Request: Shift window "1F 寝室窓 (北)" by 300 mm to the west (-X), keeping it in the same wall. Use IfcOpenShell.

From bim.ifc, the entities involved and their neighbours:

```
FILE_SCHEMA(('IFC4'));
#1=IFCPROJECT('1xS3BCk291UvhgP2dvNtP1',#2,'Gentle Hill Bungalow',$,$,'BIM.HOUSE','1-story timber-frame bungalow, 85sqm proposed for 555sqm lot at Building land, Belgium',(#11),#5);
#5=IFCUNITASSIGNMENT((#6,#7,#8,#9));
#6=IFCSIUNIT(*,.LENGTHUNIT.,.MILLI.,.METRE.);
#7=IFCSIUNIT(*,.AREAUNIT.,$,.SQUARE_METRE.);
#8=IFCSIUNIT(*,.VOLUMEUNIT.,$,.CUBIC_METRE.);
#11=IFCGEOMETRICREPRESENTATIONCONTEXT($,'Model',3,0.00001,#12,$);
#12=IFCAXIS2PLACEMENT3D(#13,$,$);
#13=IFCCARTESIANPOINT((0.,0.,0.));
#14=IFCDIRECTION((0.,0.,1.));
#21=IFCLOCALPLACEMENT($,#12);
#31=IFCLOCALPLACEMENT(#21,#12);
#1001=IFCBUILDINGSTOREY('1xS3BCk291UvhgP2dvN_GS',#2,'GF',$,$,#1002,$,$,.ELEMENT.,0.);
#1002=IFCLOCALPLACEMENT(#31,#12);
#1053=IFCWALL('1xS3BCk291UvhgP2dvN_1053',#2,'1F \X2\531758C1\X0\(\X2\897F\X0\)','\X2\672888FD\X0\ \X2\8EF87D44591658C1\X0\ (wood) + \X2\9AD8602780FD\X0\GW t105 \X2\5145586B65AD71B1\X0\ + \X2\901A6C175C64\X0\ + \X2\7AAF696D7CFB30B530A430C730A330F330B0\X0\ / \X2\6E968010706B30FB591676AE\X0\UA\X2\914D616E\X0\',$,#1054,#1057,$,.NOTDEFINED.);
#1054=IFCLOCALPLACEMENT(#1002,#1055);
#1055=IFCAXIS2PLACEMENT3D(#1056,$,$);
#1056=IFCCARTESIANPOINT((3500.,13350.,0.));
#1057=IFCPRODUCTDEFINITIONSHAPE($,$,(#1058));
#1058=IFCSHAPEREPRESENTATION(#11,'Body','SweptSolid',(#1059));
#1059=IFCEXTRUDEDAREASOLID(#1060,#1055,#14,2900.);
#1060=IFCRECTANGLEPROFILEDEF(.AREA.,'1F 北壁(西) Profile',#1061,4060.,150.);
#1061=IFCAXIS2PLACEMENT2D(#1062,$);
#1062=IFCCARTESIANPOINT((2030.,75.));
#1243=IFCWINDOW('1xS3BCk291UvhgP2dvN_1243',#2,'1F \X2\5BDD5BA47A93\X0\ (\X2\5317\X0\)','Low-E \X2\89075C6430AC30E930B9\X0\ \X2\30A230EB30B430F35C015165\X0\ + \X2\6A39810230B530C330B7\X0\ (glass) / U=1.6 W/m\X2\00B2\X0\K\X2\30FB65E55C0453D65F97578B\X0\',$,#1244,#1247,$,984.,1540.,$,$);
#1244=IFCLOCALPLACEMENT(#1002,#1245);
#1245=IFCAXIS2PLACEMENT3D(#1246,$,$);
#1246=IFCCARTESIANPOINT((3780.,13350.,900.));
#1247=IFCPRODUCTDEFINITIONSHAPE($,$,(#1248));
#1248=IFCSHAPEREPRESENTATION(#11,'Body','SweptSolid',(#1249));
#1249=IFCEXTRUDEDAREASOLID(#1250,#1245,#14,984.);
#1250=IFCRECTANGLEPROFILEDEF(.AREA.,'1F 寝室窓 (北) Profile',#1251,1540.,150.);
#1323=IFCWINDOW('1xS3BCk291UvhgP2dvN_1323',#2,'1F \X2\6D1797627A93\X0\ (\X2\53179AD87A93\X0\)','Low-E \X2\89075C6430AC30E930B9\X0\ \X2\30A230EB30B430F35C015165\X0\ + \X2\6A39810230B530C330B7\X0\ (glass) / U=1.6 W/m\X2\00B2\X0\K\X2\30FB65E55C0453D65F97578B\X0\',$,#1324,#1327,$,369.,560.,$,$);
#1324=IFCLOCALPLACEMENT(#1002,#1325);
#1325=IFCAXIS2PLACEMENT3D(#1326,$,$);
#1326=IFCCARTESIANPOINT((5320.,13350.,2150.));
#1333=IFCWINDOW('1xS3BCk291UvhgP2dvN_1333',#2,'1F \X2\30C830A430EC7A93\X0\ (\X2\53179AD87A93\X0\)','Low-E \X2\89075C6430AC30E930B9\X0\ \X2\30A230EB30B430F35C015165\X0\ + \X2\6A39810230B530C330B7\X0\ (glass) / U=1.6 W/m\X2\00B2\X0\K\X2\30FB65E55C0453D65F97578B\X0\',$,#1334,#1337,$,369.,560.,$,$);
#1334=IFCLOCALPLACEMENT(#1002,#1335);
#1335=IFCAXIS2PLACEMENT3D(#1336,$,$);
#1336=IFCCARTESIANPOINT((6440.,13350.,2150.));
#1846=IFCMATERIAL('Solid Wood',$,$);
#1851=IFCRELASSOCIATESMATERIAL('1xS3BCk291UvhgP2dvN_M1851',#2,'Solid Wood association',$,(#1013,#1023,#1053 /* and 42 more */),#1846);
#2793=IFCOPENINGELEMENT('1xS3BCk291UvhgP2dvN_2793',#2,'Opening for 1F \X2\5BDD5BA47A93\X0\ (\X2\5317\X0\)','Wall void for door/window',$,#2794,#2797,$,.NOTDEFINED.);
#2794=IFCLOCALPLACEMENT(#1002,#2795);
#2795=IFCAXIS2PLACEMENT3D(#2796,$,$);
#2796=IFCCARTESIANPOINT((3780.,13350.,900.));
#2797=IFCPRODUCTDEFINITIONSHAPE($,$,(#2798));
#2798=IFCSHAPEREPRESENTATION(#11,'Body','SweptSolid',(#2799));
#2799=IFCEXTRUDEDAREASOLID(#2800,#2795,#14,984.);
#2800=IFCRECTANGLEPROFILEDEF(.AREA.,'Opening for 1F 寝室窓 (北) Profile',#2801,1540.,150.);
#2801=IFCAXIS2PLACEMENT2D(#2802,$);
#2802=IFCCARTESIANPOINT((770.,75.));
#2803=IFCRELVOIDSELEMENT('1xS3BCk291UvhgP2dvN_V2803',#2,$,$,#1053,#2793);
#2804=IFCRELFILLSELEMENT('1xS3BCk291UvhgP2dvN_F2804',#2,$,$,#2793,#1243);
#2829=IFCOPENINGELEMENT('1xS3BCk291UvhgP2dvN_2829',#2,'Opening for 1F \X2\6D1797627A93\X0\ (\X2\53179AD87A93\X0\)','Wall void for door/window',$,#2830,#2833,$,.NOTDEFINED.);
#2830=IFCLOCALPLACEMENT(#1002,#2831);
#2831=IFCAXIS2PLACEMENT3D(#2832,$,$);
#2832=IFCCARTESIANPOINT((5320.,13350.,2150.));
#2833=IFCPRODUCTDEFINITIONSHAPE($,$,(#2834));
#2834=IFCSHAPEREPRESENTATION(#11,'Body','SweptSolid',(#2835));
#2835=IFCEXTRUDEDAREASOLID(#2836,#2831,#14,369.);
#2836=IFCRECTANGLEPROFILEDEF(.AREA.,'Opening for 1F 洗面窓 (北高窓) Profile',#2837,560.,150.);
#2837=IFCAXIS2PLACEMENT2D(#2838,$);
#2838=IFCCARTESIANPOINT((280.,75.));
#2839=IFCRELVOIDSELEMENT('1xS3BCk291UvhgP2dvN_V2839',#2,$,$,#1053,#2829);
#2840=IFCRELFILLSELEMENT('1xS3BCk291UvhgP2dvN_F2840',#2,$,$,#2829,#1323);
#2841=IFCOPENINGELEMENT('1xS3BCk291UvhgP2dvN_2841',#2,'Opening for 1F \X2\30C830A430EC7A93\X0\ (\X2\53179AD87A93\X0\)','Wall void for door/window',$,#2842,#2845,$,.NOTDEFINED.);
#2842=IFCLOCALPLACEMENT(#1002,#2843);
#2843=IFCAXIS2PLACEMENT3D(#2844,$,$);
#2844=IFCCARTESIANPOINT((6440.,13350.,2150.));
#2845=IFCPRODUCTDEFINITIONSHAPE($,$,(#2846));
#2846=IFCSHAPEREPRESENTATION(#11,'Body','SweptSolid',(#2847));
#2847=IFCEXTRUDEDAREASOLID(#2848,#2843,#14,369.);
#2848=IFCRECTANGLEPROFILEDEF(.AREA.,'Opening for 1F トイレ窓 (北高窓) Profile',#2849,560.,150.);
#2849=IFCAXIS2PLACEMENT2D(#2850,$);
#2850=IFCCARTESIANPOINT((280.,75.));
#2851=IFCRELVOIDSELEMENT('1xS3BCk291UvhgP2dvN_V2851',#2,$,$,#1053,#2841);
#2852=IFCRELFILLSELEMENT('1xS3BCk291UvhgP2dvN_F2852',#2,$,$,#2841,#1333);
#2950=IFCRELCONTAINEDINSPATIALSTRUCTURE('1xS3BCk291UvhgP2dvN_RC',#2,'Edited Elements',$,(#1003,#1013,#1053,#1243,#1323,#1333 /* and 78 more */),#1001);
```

```python
import ifcopenshell
import ifcopenshell.api.geometry
import ifcopenshell.util.placement
import ifcopenshell.util.unit

model = ifcopenshell.open("bim.ifc")
unit_scale = ifcopenshell.util.unit.calculate_unit_scale(model)

window = model.by_guid("1xS3BCk291UvhgP2dvN_1243")
opening = window.FillsVoids[0].RelatingOpeningElement
wall = opening.VoidsElements[0].RelatingBuildingElement

wall_matrix = ifcopenshell.util.placement.get_local_placement(wall.ObjectPlacement)
shift = wall_matrix[:3, 0] * -0.3 / unit_scale
before = ifcopenshell.util.placement.get_local_placement(window.ObjectPlacement)[:3, 3].copy()

# The window is not placed relative to its opening, so move both.
for product in (opening, window):
    matrix = ifcopenshell.util.placement.get_local_placement(product.ObjectPlacement)
    matrix[:3, 3] += shift
    ifcopenshell.api.geometry.edit_object_placement(model, product=product, matrix=matrix, is_si=False)

after = ifcopenshell.util.placement.get_local_placement(window.ObjectPlacement)[:3, 3]
print("window moved by", (after - before).round(3) + 0.0)

model.write("bim_rev.ifc")
```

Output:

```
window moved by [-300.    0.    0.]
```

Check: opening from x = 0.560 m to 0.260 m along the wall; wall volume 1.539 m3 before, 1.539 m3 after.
